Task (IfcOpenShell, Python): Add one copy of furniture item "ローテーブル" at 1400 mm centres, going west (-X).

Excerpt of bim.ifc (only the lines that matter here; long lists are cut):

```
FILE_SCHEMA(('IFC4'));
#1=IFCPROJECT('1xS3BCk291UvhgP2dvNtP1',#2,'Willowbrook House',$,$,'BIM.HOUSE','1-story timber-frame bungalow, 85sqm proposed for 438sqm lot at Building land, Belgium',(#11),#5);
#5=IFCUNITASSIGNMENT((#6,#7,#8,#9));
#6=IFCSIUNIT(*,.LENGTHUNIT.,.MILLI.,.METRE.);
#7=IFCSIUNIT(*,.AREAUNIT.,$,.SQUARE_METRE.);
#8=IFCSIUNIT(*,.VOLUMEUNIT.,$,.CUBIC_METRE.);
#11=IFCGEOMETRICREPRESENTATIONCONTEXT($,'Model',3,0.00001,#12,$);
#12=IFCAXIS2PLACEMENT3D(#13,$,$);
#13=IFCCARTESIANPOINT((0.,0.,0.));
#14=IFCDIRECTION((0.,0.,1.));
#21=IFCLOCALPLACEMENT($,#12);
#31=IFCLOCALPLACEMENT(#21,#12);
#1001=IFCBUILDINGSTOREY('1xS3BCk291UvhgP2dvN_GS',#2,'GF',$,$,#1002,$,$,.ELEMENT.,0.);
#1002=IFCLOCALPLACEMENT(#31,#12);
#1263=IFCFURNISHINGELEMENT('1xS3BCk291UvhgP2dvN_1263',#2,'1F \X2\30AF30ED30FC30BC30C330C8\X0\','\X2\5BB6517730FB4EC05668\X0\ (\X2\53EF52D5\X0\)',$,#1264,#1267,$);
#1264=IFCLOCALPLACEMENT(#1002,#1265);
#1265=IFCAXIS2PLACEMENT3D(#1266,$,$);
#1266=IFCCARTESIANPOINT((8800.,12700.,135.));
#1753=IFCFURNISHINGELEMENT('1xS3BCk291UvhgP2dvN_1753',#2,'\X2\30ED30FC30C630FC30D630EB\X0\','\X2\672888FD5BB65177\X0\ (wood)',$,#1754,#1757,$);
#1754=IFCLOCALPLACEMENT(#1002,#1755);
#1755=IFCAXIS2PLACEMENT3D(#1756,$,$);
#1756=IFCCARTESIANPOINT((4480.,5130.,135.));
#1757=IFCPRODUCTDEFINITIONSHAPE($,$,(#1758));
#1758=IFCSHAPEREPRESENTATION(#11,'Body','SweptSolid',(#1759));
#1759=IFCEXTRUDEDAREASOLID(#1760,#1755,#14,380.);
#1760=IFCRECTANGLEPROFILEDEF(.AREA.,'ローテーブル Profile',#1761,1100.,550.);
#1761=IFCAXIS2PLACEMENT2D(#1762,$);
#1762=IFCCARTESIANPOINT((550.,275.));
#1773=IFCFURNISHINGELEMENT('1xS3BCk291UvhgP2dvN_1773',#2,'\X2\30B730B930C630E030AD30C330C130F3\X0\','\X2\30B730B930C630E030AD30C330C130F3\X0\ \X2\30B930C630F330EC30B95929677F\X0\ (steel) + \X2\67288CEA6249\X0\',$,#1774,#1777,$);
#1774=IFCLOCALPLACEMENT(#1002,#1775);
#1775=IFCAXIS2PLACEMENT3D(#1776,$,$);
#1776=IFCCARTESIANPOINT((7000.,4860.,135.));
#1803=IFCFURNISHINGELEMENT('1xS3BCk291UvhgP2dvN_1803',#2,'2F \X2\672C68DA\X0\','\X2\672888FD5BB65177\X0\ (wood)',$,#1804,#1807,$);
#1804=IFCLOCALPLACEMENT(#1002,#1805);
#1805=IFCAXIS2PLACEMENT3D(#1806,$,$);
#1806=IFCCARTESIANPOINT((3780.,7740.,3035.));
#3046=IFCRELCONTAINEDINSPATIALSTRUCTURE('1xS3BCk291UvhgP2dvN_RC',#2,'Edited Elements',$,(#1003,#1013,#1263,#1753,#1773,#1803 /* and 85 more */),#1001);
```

```python
import numpy as np
import ifcopenshell
import ifcopenshell.api.geometry
import ifcopenshell.api.root
import ifcopenshell.util.element
import ifcopenshell.util.placement
import ifcopenshell.util.unit

model = ifcopenshell.open("bim.ifc")
unit_scale = ifcopenshell.util.unit.calculate_unit_scale(model)


def reuse_history(source, copy):
    """copy_class also copies each property set's owner history, people and application; keep the originals."""
    for rel in copy.IsDefinedBy:
        if rel.is_a("IfcRelDefinesByProperties") and (history := rel.RelatingPropertyDefinition.OwnerHistory):
            rel.RelatingPropertyDefinition.OwnerHistory = source.OwnerHistory
            ifcopenshell.util.element.remove_deep2(model, history)


source = model.by_id(1753)
base = ifcopenshell.util.placement.get_local_placement(source.ObjectPlacement)
step = np.array([-1.0, 0.0, 0.0]) * 1.4 / unit_scale

for i in range(1, 2):
    copy = ifcopenshell.api.root.copy_class(model, product=source)
    copy.Representation = ifcopenshell.util.element.copy_deep(
        model, source.Representation, exclude=["IfcGeometricRepresentationContext", "IfcRepresentationMap"]
    )
    reuse_history(source, copy)
    matrix = base.copy()
    matrix[:3, 3] += i * step
    print("added at", matrix[:3, 3].round(3) + 0.0)
    ifcopenshell.api.geometry.edit_object_placement(model, product=copy, matrix=matrix, is_si=False)

model.write("bim_updated.ifc")
```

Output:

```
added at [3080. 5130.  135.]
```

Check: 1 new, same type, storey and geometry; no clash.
